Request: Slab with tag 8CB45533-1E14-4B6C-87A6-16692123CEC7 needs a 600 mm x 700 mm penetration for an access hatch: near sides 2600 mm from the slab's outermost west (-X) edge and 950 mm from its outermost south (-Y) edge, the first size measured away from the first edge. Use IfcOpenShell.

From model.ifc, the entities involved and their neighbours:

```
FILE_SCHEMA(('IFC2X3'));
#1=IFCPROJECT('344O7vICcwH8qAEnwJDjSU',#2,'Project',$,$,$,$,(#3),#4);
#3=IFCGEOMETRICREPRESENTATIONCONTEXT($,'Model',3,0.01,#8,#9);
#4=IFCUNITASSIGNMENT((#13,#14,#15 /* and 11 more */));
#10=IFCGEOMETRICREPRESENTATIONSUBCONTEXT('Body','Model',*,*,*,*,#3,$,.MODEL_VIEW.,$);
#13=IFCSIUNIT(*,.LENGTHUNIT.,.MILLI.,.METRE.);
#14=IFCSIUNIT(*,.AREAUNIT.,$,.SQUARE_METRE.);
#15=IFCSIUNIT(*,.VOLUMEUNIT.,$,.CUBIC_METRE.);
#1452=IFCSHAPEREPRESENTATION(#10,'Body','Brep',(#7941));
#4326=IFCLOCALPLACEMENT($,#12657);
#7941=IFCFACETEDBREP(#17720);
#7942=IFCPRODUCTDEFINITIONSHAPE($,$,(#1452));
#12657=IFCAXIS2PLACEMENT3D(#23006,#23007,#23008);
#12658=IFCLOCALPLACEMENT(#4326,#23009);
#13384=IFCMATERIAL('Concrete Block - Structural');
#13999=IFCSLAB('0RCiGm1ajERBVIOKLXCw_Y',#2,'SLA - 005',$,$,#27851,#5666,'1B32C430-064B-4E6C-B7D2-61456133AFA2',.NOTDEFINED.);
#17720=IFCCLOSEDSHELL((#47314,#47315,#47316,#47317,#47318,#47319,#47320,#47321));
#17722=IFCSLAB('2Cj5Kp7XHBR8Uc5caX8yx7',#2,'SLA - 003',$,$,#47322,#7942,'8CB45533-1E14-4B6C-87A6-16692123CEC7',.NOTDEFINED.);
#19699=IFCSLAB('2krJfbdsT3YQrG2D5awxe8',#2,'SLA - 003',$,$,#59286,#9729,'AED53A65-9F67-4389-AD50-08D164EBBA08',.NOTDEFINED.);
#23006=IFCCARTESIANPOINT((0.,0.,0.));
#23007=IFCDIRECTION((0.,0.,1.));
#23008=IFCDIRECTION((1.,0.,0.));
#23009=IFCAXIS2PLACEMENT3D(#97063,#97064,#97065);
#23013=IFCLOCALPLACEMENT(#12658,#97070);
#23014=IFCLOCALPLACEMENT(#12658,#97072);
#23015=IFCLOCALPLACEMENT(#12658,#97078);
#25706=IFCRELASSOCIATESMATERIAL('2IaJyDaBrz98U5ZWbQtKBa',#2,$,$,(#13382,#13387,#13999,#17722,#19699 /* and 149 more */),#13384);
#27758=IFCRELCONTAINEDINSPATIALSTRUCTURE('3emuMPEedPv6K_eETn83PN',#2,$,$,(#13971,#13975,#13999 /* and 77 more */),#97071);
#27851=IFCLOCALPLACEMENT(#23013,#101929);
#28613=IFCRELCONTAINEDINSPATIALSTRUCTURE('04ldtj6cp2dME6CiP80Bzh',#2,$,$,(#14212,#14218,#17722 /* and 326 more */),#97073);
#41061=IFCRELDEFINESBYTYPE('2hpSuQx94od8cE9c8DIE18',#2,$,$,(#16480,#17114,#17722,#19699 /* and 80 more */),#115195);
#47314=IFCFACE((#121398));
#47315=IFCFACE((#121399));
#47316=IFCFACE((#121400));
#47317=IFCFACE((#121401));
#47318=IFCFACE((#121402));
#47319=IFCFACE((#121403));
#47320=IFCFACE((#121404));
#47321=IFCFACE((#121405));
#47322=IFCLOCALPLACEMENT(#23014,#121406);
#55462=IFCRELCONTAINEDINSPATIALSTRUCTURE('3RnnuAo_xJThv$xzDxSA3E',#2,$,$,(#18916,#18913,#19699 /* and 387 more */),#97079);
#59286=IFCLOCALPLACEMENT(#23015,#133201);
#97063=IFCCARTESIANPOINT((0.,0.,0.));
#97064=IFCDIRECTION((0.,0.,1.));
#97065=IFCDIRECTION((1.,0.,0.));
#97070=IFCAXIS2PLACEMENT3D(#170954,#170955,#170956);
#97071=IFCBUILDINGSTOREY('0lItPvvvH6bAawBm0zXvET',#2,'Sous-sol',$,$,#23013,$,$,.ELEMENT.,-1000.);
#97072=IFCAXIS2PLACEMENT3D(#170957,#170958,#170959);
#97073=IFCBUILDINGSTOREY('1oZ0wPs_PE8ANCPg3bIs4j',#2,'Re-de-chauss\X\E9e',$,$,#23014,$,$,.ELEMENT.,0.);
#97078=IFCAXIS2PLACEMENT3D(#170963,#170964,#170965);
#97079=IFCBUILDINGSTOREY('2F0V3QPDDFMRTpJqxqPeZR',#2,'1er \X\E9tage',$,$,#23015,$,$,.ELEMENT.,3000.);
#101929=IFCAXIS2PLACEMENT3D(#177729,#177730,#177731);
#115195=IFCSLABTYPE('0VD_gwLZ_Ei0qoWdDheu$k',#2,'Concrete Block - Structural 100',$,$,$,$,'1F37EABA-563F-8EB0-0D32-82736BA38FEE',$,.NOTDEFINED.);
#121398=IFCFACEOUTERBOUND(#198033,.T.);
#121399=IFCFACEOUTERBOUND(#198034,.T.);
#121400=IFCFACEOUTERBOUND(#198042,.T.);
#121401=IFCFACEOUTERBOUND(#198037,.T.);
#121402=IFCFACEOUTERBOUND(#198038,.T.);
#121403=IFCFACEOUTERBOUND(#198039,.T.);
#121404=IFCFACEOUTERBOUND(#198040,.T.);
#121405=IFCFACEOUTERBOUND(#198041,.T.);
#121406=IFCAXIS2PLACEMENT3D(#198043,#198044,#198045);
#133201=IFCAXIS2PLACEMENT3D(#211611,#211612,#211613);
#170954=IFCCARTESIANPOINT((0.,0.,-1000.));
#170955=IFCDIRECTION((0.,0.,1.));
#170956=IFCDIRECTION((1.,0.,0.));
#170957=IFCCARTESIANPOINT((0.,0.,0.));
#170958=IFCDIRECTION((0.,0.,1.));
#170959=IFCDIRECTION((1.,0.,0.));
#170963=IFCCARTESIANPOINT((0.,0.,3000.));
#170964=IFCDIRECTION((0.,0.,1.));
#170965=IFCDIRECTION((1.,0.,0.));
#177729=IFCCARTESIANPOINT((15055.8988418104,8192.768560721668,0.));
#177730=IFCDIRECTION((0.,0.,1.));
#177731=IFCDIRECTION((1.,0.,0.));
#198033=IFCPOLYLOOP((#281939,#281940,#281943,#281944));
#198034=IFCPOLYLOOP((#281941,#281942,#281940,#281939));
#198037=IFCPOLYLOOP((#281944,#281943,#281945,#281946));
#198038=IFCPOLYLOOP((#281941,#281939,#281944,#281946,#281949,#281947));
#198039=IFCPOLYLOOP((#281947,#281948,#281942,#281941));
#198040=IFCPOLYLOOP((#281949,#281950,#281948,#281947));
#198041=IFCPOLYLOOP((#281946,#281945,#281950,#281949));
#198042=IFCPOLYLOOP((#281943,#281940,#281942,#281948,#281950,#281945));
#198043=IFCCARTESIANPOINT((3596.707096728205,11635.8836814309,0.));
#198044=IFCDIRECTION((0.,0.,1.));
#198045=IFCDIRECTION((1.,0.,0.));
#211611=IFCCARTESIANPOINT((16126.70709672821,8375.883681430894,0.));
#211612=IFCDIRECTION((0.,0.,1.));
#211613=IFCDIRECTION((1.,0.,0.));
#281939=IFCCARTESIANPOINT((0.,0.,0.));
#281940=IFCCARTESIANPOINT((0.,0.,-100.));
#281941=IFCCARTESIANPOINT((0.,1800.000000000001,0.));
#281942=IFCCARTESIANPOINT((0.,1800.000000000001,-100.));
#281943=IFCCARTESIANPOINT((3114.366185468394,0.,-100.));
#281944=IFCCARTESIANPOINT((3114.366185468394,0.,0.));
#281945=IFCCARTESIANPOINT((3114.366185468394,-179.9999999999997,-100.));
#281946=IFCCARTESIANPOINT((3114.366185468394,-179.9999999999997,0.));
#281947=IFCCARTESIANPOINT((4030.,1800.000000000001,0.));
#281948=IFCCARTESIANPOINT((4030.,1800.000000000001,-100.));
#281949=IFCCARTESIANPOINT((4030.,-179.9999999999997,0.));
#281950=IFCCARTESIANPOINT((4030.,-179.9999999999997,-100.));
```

```python
import numpy as np
import ifcopenshell
import ifcopenshell.api.feature
import ifcopenshell.api.geometry
import ifcopenshell.api.root
import ifcopenshell.geom
import ifcopenshell.util.placement
import ifcopenshell.util.representation
import ifcopenshell.util.shape
import ifcopenshell.util.unit

model = ifcopenshell.open("model.ifc")
unit_scale = ifcopenshell.util.unit.calculate_unit_scale(model)
settings = ifcopenshell.geom.settings()


def volume(element):
    """Net volume in cubic metres, openings subtracted."""
    shape = ifcopenshell.geom.create_shape(settings, element)
    return ifcopenshell.util.shape.get_volume(shape.geometry)


slab = model.by_guid("2Cj5Kp7XHBR8Uc5caX8yx7")
before = volume(slab)

# Extent in the slab's own axes, in metres. The edges named are its -X and -Y sides.
slab_shape = ifcopenshell.geom.create_shape(settings, slab)
vertices = ifcopenshell.util.shape.get_vertices(slab_shape.geometry)
x_min, y_min, bottom = vertices.min(axis=0)
top = vertices[:, 2].max()

opening = ifcopenshell.api.root.create_entity(model, ifc_class="IfcOpeningElement", name="Access hatch opening")
context = ifcopenshell.util.representation.get_context(model, "Model", "Body", "MODEL_VIEW")
width, depth = 0.6, 0.7
outline = [(0.0, 0.0), (width, 0.0), (width, depth), (0.0, depth), (0.0, 0.0)]
# Overshoot both faces by 50 mm so the cut is clean.
shape = ifcopenshell.api.geometry.add_slab_representation(
    model, context=context, depth=top - bottom + 0.1, polyline=outline
)
ifcopenshell.api.geometry.assign_representation(model, product=opening, representation=shape)

matrix = ifcopenshell.util.placement.get_local_placement(slab.ObjectPlacement)
matrix[:, 3] = matrix @ np.append(np.array([x_min + 2.6, y_min + 0.95, bottom - 0.05]) / unit_scale, 1.0)
ifcopenshell.api.geometry.edit_object_placement(model, product=opening, matrix=matrix, is_si=False)
ifcopenshell.api.feature.add_feature(model, feature=opening, element=slab)

after = volume(slab)

print(f"slab volume {before:.3f} -> {after:.3f} m3")

model.write("model_edited.ifc")
```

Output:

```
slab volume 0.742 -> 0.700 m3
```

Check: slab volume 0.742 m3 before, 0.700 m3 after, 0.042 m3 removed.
